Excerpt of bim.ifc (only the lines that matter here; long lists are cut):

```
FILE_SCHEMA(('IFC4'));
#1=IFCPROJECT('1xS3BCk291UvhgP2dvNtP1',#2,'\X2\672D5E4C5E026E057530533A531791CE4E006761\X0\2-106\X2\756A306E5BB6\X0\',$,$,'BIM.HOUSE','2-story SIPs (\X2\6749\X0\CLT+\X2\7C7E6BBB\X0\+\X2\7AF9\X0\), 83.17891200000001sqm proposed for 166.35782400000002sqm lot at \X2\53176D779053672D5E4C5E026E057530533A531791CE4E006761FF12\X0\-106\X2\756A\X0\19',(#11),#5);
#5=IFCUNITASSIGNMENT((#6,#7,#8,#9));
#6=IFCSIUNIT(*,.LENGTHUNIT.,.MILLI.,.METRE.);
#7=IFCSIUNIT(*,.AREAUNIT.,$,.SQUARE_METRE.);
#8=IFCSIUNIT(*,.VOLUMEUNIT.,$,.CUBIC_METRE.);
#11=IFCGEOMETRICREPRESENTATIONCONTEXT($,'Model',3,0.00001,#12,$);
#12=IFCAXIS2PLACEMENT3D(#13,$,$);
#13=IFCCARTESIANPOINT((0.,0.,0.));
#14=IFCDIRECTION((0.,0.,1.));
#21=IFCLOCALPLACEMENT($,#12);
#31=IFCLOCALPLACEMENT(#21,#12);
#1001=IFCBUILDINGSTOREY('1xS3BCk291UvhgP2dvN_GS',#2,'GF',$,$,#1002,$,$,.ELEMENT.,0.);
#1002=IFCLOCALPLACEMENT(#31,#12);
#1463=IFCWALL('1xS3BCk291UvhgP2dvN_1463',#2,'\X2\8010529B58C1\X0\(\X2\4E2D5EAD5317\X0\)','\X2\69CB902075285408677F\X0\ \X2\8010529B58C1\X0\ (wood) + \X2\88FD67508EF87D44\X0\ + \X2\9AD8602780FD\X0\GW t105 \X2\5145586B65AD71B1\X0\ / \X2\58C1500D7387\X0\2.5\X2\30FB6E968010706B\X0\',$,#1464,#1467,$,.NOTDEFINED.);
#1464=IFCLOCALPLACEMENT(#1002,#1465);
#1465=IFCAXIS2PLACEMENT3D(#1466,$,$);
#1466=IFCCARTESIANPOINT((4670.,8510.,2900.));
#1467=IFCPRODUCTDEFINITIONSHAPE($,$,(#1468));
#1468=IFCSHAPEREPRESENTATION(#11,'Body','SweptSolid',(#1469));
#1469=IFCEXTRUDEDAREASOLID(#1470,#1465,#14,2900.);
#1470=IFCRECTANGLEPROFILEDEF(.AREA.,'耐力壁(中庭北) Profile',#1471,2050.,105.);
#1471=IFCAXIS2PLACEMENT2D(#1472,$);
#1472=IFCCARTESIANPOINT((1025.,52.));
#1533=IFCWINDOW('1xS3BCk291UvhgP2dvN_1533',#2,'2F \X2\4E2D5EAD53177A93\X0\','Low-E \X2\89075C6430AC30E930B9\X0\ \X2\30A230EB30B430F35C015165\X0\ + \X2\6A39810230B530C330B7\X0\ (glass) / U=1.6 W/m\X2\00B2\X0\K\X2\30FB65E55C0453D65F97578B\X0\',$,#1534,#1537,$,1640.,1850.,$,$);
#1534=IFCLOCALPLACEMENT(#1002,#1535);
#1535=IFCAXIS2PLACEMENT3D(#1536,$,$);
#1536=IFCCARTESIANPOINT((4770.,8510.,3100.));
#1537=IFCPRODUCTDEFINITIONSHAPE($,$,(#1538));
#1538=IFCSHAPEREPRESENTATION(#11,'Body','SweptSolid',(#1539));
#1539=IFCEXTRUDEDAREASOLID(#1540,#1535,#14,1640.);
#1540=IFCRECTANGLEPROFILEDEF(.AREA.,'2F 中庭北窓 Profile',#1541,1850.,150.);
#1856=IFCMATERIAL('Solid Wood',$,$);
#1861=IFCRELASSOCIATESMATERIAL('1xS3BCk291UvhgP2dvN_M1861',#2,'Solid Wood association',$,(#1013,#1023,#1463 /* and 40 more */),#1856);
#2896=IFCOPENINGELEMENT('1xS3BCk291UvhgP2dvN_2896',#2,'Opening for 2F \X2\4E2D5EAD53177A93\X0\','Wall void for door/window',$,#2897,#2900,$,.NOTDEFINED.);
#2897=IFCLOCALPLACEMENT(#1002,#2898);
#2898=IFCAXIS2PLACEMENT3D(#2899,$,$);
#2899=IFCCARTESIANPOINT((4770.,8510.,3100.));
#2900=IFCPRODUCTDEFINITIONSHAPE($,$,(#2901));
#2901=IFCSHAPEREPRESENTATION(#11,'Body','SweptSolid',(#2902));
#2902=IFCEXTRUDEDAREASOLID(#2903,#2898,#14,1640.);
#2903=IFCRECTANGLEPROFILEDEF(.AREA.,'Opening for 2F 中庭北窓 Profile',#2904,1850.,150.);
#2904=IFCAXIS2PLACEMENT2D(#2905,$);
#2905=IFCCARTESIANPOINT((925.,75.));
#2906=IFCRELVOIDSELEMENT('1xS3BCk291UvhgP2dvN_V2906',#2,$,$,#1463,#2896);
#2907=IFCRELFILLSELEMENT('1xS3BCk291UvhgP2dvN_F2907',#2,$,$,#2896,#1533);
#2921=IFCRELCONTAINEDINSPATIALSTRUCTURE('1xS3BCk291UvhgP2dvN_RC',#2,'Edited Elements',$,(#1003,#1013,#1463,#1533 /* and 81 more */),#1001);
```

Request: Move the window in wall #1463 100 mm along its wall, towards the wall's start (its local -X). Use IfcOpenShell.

```python
import ifcopenshell
import ifcopenshell.api.geometry
import ifcopenshell.util.placement
import ifcopenshell.util.unit

model = ifcopenshell.open("bim.ifc")
unit_scale = ifcopenshell.util.unit.calculate_unit_scale(model)

window = model.by_guid("1xS3BCk291UvhgP2dvN_1533")
opening = window.FillsVoids[0].RelatingOpeningElement
wall = opening.VoidsElements[0].RelatingBuildingElement

wall_matrix = ifcopenshell.util.placement.get_local_placement(wall.ObjectPlacement)
shift = wall_matrix[:3, 0] * -0.1 / unit_scale
before = ifcopenshell.util.placement.get_local_placement(window.ObjectPlacement)[:3, 3].copy()

# The window is not placed relative to its opening, so move both.
for product in (opening, window):
    matrix = ifcopenshell.util.placement.get_local_placement(product.ObjectPlacement)
    matrix[:3, 3] += shift
    ifcopenshell.api.geometry.edit_object_placement(model, product=product, matrix=matrix, is_si=False)

after = ifcopenshell.util.placement.get_local_placement(window.ObjectPlacement)[:3, 3]
print("window moved by", (after - before).round(3) + 0.0)

model.write("bim_edited.ifc")
```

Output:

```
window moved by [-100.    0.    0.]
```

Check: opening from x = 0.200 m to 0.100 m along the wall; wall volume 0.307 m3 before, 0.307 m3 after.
